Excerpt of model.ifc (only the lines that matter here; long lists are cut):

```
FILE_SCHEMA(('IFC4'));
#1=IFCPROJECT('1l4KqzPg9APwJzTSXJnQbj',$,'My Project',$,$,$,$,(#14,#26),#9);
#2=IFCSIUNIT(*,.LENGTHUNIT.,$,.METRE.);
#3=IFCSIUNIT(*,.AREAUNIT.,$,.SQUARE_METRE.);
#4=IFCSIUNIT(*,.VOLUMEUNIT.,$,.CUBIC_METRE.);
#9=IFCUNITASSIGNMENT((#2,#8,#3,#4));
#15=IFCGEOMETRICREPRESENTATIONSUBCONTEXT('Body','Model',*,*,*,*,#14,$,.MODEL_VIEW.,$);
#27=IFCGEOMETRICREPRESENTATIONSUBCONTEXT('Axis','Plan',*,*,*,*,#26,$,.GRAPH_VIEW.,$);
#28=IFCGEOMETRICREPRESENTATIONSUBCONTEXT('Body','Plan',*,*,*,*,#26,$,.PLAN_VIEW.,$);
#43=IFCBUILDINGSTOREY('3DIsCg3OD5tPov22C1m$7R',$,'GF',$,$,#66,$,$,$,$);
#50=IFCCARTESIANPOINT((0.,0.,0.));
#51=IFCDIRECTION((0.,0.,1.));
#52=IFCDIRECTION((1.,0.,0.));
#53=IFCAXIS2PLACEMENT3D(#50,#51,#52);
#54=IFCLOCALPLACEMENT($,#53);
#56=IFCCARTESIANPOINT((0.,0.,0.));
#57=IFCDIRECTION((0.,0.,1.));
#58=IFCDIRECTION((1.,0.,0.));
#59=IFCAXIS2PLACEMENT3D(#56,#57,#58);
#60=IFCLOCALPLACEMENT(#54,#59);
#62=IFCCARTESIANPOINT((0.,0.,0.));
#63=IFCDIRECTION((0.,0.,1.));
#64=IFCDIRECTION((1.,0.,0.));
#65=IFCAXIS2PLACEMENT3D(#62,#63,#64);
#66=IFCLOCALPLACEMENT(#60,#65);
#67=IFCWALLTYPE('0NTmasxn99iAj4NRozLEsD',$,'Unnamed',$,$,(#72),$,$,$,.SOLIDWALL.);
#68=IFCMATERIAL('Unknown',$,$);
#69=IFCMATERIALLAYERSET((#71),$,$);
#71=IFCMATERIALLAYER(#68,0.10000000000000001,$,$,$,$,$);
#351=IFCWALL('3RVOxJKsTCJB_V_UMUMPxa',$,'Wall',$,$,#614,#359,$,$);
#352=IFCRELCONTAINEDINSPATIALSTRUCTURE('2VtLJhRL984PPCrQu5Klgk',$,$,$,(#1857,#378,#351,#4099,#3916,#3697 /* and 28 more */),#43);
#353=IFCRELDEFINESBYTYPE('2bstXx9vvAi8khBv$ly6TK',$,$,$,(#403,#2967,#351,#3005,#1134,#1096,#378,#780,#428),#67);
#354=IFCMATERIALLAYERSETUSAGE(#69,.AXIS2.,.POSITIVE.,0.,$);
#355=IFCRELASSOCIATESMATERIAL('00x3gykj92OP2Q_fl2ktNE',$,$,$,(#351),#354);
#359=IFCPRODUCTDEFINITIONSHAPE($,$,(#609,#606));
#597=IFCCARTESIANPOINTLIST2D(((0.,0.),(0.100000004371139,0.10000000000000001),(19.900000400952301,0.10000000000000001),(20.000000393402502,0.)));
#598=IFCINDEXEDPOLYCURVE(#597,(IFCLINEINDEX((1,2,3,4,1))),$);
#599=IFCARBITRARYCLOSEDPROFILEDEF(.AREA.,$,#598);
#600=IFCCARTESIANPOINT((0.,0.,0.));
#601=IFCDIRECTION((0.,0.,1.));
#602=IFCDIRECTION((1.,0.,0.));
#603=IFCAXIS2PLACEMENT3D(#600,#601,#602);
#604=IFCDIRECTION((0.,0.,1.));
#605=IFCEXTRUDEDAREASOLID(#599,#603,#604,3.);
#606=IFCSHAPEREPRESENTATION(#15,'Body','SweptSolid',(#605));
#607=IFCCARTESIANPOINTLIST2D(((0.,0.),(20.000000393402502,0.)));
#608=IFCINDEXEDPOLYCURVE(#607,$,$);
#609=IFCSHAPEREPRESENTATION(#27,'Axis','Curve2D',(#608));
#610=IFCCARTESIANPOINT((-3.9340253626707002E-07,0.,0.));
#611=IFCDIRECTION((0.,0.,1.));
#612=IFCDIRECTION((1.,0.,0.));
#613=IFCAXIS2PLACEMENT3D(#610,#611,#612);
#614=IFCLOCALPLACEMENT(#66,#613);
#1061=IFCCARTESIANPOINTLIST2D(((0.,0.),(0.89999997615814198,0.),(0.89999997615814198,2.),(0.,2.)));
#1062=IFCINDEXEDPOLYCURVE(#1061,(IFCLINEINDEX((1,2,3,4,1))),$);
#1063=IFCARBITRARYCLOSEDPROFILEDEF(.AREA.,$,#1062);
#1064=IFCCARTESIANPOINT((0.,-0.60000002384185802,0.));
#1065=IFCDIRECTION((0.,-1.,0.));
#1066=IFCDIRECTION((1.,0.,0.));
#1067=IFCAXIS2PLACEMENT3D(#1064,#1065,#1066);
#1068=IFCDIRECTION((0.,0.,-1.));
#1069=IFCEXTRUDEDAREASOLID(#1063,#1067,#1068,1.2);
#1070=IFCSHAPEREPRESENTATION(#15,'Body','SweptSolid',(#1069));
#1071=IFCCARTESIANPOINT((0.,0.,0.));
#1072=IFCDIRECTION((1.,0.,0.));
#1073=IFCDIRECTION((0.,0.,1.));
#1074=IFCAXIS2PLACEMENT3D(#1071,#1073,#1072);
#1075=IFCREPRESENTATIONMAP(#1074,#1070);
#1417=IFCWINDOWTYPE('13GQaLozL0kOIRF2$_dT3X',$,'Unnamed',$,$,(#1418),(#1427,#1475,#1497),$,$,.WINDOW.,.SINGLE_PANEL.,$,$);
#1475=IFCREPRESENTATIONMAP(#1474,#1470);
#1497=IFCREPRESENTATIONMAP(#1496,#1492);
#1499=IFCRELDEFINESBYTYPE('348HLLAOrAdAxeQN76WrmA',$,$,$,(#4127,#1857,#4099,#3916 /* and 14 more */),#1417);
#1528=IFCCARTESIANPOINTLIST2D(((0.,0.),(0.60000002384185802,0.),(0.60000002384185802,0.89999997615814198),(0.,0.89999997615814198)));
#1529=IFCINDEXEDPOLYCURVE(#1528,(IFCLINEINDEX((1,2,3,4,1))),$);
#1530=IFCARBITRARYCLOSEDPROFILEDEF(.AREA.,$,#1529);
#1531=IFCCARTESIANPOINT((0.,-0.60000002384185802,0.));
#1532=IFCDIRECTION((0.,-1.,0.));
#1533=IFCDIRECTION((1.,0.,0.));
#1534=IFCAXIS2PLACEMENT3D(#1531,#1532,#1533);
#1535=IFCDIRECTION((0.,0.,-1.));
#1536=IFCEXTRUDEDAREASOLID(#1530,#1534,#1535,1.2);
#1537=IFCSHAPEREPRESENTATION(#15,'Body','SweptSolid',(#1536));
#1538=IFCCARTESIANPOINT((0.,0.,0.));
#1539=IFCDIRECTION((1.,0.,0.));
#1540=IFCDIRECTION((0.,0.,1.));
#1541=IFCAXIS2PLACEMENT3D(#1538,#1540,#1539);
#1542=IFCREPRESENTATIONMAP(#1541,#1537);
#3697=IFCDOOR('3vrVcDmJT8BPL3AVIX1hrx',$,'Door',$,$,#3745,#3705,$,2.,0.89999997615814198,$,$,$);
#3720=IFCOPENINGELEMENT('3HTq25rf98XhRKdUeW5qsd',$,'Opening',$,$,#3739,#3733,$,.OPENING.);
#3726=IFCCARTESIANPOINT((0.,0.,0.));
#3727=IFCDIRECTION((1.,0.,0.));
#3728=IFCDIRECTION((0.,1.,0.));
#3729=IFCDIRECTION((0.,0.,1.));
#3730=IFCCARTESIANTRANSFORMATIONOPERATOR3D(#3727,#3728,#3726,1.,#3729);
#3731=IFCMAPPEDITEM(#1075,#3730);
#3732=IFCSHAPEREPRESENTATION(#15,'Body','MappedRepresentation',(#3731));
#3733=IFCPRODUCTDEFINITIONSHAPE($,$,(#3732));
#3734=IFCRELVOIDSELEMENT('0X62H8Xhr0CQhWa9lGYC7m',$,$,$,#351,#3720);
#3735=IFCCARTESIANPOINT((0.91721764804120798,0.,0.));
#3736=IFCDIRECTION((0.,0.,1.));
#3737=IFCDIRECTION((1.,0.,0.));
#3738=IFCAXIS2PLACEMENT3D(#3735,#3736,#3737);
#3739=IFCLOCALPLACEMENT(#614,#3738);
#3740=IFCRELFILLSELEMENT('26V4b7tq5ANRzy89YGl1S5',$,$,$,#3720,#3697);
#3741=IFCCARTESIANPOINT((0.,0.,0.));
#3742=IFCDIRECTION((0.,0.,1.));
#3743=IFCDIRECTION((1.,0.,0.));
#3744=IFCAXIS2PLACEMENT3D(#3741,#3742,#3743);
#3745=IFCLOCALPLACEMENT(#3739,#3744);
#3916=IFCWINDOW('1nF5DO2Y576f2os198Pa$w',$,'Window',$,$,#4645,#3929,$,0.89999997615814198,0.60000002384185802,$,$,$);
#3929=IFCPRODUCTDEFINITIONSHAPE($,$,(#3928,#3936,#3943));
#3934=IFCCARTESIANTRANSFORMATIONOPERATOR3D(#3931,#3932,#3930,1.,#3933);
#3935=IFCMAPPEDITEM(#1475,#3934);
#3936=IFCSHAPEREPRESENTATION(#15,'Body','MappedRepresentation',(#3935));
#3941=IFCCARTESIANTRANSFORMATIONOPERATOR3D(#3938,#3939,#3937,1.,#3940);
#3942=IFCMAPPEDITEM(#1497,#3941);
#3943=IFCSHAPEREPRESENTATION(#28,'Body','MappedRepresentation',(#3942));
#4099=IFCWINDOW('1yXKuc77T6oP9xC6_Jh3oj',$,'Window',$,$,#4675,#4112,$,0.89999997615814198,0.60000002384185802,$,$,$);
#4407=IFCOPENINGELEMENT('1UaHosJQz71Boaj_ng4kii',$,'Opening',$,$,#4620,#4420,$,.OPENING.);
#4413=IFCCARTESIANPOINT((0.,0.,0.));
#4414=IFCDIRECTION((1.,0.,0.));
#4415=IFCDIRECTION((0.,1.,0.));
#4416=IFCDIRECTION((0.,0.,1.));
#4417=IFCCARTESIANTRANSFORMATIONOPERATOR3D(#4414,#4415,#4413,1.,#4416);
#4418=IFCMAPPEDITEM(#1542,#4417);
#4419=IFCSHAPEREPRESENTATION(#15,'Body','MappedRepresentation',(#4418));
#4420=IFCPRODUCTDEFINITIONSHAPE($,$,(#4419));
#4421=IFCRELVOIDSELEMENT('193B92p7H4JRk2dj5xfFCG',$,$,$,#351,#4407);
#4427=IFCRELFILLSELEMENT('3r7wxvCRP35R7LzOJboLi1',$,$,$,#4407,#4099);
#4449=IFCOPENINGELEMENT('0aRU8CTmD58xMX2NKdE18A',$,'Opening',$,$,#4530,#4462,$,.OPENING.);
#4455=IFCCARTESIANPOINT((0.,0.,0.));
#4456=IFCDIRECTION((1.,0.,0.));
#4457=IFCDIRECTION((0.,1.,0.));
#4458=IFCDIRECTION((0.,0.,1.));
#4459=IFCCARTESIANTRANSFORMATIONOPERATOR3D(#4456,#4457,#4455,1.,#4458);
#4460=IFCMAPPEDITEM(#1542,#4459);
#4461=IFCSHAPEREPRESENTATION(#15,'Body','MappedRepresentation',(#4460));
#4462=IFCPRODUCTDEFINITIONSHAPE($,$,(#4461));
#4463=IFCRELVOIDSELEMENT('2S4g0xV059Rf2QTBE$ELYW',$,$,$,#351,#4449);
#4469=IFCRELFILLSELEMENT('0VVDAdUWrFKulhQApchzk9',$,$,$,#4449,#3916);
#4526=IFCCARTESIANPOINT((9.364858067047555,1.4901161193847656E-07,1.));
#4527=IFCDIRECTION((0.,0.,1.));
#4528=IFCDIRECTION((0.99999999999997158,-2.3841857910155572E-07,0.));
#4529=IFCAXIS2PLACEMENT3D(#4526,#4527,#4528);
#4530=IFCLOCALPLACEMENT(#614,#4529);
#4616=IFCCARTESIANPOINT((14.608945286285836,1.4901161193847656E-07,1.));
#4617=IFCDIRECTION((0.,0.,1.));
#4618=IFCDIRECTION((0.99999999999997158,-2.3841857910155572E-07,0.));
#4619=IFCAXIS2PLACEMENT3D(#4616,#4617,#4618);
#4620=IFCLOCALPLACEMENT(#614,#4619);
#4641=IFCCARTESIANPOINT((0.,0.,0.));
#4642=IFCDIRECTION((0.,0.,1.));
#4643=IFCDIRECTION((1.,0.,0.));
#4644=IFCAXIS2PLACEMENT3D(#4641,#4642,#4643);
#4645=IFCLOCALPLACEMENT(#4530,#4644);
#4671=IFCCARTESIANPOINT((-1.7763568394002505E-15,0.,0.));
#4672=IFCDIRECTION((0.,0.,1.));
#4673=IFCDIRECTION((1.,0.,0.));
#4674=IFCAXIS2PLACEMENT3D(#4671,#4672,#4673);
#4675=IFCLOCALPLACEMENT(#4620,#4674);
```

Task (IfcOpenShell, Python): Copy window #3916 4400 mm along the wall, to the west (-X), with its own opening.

```python
import ifcopenshell
import ifcopenshell.api.feature
import ifcopenshell.api.geometry
import ifcopenshell.api.root
import ifcopenshell.geom
import ifcopenshell.util.element
import ifcopenshell.util.placement
import ifcopenshell.util.shape
import ifcopenshell.util.unit

model = ifcopenshell.open("model.ifc")
unit_scale = ifcopenshell.util.unit.calculate_unit_scale(model)
settings = ifcopenshell.geom.settings()


def volume(element):
    """Net volume in cubic metres, openings subtracted."""
    shape = ifcopenshell.geom.create_shape(settings, element)
    return ifcopenshell.util.shape.get_volume(shape.geometry)


window = model.by_guid("1nF5DO2Y576f2os198Pa$w")
opening = window.FillsVoids[0].RelatingOpeningElement
wall = opening.VoidsElements[0].RelatingBuildingElement
before = volume(wall)
shift = ifcopenshell.util.placement.get_local_placement(wall.ObjectPlacement)[:3, 0] * -4.4 / unit_scale

# copy_class copies the void relationship, type, container and properties, but no geometry.
new_opening = ifcopenshell.api.root.copy_class(model, product=opening)
new_opening.Representation = ifcopenshell.util.element.copy_deep(
    model, opening.Representation, exclude=["IfcGeometricRepresentationContext", "IfcRepresentationMap"]
)
new_window = ifcopenshell.api.root.copy_class(model, product=window)
new_window.Representation = ifcopenshell.util.element.copy_deep(
    model, window.Representation, exclude=["IfcGeometricRepresentationContext", "IfcRepresentationMap"]
)
ifcopenshell.api.feature.add_filling(model, opening=new_opening, element=new_window)

for old, new in ((opening, new_opening), (window, new_window)):
    matrix = ifcopenshell.util.placement.get_local_placement(old.ObjectPlacement)
    matrix[:3, 3] += shift
    ifcopenshell.api.geometry.edit_object_placement(model, product=new, matrix=matrix, is_si=False)

after = volume(wall)

print(f"wall volume {before:.3f} -> {after:.3f} m3")

model.write("model_edited.ifc")
```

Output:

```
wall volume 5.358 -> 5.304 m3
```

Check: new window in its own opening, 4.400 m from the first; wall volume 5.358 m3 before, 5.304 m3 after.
